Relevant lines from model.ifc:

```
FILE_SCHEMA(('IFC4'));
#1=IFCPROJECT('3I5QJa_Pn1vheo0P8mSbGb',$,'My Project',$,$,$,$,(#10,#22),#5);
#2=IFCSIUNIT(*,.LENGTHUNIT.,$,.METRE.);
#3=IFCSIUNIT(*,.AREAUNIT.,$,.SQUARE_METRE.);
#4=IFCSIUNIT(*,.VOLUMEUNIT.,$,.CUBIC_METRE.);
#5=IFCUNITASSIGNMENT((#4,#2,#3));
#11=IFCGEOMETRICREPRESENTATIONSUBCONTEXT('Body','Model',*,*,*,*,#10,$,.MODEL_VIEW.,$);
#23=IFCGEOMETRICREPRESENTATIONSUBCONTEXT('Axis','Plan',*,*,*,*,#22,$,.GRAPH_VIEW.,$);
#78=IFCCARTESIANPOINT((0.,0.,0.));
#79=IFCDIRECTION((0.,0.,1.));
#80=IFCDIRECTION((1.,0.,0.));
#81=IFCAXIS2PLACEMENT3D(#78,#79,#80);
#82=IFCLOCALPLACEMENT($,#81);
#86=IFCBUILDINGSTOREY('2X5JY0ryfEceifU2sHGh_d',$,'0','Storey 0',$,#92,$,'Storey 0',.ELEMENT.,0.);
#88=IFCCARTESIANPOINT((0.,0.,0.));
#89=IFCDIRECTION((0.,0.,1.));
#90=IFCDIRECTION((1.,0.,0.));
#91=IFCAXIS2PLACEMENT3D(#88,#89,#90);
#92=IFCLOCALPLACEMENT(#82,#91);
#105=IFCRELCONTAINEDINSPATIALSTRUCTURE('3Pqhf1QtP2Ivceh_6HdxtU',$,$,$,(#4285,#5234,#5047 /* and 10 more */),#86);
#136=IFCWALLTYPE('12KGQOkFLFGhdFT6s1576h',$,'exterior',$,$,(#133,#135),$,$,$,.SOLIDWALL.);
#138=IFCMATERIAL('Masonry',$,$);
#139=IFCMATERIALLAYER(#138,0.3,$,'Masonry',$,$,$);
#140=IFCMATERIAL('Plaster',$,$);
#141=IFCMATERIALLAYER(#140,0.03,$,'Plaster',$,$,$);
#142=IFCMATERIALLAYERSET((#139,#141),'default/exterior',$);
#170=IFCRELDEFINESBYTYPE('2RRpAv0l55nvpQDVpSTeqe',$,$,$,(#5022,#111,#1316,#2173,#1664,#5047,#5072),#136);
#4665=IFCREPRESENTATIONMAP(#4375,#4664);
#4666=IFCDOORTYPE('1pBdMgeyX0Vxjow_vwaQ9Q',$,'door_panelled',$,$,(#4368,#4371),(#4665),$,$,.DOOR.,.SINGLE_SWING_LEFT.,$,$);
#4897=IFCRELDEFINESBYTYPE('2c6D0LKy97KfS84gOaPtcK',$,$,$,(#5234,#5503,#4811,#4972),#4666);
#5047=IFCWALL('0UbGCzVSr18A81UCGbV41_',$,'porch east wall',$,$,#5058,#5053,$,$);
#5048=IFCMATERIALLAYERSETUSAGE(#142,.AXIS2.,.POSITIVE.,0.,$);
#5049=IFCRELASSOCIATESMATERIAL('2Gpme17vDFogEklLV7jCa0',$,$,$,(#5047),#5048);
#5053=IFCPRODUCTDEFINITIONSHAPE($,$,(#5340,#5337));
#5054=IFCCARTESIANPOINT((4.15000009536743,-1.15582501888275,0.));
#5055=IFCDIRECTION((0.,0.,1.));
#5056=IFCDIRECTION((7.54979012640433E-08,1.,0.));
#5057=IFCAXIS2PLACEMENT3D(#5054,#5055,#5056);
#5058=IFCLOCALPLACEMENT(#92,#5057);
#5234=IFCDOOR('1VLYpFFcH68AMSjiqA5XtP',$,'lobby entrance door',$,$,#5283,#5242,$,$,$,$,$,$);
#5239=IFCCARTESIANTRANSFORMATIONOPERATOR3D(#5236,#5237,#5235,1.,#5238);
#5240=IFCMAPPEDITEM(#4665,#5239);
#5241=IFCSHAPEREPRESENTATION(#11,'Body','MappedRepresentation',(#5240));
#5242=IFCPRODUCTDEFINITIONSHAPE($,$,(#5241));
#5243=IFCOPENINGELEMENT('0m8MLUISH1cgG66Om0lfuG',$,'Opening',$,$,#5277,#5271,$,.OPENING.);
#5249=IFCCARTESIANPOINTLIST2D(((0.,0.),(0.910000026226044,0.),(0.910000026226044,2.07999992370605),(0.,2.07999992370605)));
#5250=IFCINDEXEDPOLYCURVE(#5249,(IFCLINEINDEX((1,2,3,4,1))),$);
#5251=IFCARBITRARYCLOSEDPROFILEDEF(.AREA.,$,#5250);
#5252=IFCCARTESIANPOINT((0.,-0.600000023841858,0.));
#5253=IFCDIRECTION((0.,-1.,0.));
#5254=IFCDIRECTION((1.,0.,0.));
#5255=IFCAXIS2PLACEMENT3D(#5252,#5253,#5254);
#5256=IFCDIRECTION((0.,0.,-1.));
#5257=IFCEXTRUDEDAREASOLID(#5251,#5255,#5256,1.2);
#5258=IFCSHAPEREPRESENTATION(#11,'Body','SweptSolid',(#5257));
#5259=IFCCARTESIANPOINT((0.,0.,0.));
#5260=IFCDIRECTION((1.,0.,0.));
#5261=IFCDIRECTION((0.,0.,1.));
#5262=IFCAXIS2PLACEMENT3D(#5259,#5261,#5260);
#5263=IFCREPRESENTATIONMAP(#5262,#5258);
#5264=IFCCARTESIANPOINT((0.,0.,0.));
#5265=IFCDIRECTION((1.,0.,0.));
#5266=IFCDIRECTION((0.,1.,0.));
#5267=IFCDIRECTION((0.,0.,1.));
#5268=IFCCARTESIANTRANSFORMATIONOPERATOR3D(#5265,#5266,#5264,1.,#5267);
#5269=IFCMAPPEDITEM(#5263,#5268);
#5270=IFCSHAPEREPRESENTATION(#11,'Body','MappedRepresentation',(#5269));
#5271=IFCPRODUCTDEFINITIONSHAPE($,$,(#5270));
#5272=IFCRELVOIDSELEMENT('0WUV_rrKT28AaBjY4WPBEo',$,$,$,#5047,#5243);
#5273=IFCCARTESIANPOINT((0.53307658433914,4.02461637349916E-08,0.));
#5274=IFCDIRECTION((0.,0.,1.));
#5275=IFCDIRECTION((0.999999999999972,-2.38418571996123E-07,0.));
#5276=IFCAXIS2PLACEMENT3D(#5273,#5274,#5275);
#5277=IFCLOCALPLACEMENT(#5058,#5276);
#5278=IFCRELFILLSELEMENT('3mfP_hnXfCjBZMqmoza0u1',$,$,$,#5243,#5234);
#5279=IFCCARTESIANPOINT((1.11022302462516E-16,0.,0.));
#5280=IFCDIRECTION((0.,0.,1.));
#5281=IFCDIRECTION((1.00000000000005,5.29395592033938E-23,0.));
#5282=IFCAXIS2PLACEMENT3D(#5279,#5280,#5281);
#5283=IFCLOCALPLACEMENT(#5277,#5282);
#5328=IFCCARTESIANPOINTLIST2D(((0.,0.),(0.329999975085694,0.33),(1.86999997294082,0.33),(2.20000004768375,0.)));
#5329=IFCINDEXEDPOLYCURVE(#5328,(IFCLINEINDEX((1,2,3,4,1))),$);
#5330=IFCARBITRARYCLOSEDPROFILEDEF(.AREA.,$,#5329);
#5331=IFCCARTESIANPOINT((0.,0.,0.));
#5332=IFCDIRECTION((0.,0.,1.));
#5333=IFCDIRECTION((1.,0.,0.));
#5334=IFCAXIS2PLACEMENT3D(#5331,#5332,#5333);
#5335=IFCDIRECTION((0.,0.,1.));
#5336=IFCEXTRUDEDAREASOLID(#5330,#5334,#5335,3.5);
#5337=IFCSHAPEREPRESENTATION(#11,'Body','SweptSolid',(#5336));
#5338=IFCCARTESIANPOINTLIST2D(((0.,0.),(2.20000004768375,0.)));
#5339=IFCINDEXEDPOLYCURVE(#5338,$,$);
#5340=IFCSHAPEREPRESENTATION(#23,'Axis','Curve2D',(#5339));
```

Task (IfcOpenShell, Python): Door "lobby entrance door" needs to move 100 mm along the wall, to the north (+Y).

```python
import ifcopenshell
import ifcopenshell.api.geometry
import ifcopenshell.util.placement

model = ifcopenshell.open("model.ifc")

door = model.by_id(5234)
opening = door.FillsVoids[0].RelatingOpeningElement
wall = opening.VoidsElements[0].RelatingBuildingElement

wall_matrix = ifcopenshell.util.placement.get_local_placement(wall.ObjectPlacement)
shift = wall_matrix[:3, 0] * 0.1
before = ifcopenshell.util.placement.get_local_placement(door.ObjectPlacement)[:3, 3].copy()

# The door is placed relative to its opening, so it follows when the opening moves.
matrix = ifcopenshell.util.placement.get_local_placement(opening.ObjectPlacement)
matrix[:3, 3] += shift
ifcopenshell.api.geometry.edit_object_placement(
    model, product=opening, matrix=matrix, is_si=False, should_transform_children=True
)

after = ifcopenshell.util.placement.get_local_placement(door.ObjectPlacement)[:3, 3]
print("door moved by", (after - before).round(3) + 0.0)

model.write("model_updated.ifc")
```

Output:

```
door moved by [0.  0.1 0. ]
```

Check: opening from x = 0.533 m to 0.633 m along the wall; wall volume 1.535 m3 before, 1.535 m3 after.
